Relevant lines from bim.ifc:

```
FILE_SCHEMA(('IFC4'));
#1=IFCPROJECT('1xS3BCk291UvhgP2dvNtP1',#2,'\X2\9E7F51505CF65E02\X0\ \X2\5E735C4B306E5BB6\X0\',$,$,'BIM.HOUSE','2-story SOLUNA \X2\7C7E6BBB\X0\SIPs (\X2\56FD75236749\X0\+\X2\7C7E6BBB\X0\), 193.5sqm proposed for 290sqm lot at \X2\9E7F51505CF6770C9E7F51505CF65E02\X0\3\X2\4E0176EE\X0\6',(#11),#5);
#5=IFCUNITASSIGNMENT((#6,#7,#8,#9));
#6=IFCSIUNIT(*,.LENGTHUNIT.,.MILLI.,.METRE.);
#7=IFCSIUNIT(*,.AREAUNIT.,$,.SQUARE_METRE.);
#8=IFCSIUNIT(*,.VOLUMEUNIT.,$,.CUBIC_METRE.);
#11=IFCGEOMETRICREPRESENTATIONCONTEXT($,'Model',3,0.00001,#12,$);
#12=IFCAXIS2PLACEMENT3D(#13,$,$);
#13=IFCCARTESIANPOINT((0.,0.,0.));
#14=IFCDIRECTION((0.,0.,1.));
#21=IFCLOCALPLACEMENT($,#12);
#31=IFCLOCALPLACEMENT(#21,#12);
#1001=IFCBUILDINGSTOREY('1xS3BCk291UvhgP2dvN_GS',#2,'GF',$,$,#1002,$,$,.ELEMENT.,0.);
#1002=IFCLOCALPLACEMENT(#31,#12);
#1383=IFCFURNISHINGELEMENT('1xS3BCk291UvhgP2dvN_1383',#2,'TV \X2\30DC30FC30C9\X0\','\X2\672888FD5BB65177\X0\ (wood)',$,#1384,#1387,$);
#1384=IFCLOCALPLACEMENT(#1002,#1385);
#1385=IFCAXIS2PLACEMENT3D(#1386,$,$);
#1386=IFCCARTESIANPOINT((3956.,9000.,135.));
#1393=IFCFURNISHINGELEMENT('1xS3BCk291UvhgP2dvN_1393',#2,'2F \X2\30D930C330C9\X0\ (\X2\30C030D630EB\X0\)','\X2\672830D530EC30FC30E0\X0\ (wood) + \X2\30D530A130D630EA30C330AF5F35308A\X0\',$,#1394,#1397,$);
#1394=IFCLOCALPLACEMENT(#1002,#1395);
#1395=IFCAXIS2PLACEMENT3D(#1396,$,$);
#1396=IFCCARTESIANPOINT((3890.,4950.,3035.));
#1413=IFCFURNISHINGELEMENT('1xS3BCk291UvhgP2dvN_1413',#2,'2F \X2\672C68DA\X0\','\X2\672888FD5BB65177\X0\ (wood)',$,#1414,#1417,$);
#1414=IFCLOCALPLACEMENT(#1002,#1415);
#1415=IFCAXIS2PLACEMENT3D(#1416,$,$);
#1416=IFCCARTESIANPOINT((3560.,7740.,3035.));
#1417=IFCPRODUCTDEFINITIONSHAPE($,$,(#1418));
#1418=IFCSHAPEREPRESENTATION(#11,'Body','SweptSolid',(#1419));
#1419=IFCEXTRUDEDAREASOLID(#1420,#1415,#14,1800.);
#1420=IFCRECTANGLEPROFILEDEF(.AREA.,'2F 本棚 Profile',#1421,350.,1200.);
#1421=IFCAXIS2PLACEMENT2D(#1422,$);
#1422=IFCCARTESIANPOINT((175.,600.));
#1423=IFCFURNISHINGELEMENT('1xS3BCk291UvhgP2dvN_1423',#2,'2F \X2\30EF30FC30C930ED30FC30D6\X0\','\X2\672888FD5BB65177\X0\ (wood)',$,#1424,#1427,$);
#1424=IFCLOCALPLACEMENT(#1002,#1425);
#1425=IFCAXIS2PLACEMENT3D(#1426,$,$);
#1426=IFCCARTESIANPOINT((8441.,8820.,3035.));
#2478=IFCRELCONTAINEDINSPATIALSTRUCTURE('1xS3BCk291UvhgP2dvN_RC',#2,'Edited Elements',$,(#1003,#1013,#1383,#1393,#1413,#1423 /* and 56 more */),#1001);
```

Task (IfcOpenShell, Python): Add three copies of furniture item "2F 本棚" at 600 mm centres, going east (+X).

```python
import numpy as np
import ifcopenshell
import ifcopenshell.api.geometry
import ifcopenshell.api.root
import ifcopenshell.util.element
import ifcopenshell.util.placement
import ifcopenshell.util.unit

model = ifcopenshell.open("bim.ifc")
unit_scale = ifcopenshell.util.unit.calculate_unit_scale(model)


def reuse_history(source, copy):
    """copy_class also copies each property set's owner history, people and application; keep the originals."""
    for rel in copy.IsDefinedBy:
        if rel.is_a("IfcRelDefinesByProperties") and (history := rel.RelatingPropertyDefinition.OwnerHistory):
            rel.RelatingPropertyDefinition.OwnerHistory = source.OwnerHistory
            ifcopenshell.util.element.remove_deep2(model, history)


source = model.by_id(1413)
base = ifcopenshell.util.placement.get_local_placement(source.ObjectPlacement)
step = np.array([1.0, 0.0, 0.0]) * 0.6 / unit_scale

for i in range(1, 4):
    copy = ifcopenshell.api.root.copy_class(model, product=source)
    copy.Representation = ifcopenshell.util.element.copy_deep(
        model, source.Representation, exclude=["IfcGeometricRepresentationContext", "IfcRepresentationMap"]
    )
    reuse_history(source, copy)
    matrix = base.copy()
    matrix[:3, 3] += i * step
    print("added at", matrix[:3, 3].round(3) + 0.0)
    ifcopenshell.api.geometry.edit_object_placement(model, product=copy, matrix=matrix, is_si=False)

model.write("bim_edited.ifc")
```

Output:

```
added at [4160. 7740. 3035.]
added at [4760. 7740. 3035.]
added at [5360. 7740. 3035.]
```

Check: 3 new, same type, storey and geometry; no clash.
